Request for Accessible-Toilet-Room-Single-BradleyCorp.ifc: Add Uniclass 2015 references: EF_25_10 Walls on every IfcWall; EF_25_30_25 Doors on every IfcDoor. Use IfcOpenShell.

First a look at what the model holds.

```python
import ifcopenshell

model = ifcopenshell.open("Accessible-Toilet-Room-Single-BradleyCorp.ifc")
print(model.schema)
print("classifications:", [c.Name for c in model.by_type("IfcClassification")])
for ifc_class in ("IfcDoor", "IfcRoof", "IfcStair", "IfcWall", "IfcWindow"):
    print(ifc_class, len(model.by_type(ifc_class)))
```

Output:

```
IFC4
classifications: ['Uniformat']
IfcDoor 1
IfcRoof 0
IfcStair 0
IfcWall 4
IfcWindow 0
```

```python
import ifcopenshell
import ifcopenshell.api.classification

model = ifcopenshell.open("Accessible-Toilet-Room-Single-BradleyCorp.ifc")

system = ifcopenshell.api.classification.add_classification(model, classification="Uniclass 2015")

codes = {
    "IfcWall": ("EF_25_10", "Walls"),
    "IfcDoor": ("EF_25_30_25", "Doors"),
}
for ifc_class, (code, name) in codes.items():
    products = model.by_type(ifc_class)
    ifcopenshell.api.classification.add_reference(
        model, products=products, classification=system, identification=code, name=name
    )
    print(code, len(products))

model.write("Accessible-Toilet-Room-Single-BradleyCorp_updated.ifc")
```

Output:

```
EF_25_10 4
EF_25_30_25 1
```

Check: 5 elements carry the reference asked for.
